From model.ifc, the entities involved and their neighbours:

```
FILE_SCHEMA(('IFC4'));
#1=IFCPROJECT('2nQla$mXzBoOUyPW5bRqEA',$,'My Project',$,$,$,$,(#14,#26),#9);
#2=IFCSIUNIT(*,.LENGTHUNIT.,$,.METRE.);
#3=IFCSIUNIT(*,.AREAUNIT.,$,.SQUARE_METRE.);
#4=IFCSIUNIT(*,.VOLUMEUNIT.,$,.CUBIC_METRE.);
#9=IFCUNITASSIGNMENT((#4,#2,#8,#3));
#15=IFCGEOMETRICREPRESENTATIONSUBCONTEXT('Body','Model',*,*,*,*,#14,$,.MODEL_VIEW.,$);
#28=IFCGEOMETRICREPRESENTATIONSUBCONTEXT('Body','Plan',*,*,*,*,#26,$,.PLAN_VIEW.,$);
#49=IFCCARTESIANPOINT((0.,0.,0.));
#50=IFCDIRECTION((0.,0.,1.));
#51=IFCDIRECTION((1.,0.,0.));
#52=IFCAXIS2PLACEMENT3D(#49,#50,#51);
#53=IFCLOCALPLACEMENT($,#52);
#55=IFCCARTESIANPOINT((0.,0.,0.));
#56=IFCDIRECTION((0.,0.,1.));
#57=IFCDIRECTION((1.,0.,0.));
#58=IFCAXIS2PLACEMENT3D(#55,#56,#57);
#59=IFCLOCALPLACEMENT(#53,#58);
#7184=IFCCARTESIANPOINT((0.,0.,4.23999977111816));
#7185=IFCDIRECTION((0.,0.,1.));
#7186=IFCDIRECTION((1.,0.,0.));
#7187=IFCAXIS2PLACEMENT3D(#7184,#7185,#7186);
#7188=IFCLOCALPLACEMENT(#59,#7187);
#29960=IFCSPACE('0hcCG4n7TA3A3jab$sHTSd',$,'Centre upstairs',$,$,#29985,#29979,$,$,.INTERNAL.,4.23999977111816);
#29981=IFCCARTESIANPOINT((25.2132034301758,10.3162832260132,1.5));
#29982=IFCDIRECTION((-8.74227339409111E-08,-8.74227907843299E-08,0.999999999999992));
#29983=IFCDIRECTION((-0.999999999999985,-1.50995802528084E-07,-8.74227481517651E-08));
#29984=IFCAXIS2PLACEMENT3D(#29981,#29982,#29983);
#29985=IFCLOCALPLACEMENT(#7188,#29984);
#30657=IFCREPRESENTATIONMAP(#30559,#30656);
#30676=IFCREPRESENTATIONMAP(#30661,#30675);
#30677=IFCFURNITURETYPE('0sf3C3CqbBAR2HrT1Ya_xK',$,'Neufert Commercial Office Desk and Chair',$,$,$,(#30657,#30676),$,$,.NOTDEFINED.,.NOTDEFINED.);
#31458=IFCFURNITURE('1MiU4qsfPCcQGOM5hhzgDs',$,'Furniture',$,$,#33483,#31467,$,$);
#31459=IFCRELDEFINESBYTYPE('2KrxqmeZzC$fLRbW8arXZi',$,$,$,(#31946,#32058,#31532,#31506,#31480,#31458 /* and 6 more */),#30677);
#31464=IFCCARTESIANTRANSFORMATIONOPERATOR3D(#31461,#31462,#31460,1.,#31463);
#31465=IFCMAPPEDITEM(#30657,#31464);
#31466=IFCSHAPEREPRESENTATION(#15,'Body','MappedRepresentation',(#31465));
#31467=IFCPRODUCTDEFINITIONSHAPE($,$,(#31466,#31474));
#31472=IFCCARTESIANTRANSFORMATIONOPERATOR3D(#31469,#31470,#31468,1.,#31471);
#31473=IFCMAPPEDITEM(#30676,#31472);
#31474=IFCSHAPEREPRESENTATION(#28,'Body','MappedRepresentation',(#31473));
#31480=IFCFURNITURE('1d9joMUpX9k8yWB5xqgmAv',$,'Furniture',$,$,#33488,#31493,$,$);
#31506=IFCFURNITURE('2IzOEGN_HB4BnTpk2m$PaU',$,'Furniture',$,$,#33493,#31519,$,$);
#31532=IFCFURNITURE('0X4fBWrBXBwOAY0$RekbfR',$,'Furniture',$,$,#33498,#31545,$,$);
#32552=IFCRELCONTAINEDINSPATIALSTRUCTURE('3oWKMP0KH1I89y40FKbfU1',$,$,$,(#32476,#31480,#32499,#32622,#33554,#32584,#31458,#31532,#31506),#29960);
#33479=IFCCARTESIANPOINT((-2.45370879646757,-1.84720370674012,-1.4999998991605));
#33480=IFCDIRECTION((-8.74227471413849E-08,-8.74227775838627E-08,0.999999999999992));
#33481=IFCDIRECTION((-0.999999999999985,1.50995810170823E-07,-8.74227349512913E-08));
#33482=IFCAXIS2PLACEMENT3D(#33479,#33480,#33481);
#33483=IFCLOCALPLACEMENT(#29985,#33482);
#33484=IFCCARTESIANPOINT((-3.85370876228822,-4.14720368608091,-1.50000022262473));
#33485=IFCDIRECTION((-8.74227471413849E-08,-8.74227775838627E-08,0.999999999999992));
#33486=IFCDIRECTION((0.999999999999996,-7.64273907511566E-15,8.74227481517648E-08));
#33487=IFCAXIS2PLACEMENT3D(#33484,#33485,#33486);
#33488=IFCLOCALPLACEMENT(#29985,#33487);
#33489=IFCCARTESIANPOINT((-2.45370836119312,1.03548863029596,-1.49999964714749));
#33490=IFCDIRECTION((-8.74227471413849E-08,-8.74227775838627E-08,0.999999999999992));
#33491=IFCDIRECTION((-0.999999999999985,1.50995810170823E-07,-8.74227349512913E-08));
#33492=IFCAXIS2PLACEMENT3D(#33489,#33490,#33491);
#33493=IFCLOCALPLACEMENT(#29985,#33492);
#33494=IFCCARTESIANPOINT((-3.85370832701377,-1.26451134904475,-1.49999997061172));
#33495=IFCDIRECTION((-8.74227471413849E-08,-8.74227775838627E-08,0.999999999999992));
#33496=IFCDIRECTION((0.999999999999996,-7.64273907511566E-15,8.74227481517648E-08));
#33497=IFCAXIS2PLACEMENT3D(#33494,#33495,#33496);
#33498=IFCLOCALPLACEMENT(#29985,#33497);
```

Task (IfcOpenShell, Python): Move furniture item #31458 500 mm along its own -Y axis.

```python
import ifcopenshell
import ifcopenshell.api.geometry
import ifcopenshell.util.placement
import ifcopenshell.util.unit

model = ifcopenshell.open("model.ifc")
unit_scale = ifcopenshell.util.unit.calculate_unit_scale(model)

item = model.by_id(31458)
matrix = ifcopenshell.util.placement.get_local_placement(item.ObjectPlacement)
matrix[:3, 3] -= matrix[:3, 1] * 0.5 / unit_scale
ifcopenshell.api.geometry.edit_object_placement(model, product=item, matrix=matrix, is_si=False)

print(ifcopenshell.util.placement.get_local_placement(item.ObjectPlacement).round(3) + 0.0)

model.write("model_updated.ifc")
```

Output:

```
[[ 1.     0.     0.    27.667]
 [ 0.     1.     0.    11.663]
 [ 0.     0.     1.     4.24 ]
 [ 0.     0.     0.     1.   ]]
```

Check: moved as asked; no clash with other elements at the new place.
